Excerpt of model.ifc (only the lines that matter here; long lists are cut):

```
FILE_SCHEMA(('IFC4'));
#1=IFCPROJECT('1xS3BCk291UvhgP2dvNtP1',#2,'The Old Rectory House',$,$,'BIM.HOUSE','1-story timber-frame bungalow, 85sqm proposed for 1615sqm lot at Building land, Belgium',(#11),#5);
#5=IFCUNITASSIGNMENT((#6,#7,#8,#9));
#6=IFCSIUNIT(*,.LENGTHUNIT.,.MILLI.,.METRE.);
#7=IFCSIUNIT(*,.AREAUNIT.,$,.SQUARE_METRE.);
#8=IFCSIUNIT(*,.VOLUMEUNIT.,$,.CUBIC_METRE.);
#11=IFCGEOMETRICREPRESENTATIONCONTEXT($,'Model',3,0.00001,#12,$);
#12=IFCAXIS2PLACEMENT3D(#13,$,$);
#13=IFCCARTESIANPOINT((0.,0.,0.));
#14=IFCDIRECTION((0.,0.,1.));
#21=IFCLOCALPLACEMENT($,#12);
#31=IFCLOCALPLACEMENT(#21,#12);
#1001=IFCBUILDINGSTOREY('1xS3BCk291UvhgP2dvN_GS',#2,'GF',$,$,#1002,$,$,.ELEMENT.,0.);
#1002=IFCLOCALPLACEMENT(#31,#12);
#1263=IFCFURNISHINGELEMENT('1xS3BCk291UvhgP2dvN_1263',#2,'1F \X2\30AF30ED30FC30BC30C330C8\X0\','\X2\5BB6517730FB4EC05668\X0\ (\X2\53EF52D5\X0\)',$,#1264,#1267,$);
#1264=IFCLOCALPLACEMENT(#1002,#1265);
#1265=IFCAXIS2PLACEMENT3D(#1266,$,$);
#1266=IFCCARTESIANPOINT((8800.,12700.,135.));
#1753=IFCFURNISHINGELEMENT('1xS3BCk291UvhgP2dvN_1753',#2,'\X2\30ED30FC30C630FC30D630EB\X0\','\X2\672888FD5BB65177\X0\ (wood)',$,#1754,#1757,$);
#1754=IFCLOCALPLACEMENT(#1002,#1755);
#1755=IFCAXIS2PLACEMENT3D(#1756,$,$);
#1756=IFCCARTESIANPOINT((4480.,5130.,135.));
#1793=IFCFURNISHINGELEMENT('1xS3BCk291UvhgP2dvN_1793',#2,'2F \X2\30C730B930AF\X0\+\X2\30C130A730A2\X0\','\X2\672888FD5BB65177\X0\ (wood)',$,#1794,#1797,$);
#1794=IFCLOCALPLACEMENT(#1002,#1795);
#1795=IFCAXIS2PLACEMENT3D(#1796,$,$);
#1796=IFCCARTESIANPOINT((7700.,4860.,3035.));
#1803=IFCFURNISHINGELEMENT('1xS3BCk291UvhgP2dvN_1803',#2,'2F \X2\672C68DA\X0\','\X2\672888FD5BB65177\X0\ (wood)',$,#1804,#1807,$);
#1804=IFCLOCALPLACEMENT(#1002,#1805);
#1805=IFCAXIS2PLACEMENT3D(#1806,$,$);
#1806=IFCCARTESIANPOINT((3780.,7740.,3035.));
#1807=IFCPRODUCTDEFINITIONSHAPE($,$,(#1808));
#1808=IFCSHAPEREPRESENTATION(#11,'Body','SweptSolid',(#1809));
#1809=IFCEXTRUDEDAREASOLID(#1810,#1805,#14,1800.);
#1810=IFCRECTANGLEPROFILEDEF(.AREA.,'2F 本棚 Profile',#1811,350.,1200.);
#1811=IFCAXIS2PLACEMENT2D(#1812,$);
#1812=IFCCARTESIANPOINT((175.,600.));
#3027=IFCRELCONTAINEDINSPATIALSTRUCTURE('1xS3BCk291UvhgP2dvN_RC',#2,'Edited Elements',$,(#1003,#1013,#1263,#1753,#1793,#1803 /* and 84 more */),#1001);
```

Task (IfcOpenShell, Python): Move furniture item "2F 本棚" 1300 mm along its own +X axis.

```python
import ifcopenshell
import ifcopenshell.api.geometry
import ifcopenshell.util.placement
import ifcopenshell.util.unit

model = ifcopenshell.open("model.ifc")
unit_scale = ifcopenshell.util.unit.calculate_unit_scale(model)

item = model.by_guid("1xS3BCk291UvhgP2dvN_1803")
matrix = ifcopenshell.util.placement.get_local_placement(item.ObjectPlacement)
matrix[:3, 3] += matrix[:3, 0] * 1.3 / unit_scale
ifcopenshell.api.geometry.edit_object_placement(model, product=item, matrix=matrix, is_si=False)

print(ifcopenshell.util.placement.get_local_placement(item.ObjectPlacement).round(3) + 0.0)

model.write("model_updated.ifc")
```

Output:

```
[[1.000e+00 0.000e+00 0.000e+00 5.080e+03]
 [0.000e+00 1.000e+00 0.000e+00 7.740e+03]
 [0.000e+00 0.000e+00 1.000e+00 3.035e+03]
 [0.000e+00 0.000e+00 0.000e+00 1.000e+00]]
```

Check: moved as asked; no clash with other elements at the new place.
